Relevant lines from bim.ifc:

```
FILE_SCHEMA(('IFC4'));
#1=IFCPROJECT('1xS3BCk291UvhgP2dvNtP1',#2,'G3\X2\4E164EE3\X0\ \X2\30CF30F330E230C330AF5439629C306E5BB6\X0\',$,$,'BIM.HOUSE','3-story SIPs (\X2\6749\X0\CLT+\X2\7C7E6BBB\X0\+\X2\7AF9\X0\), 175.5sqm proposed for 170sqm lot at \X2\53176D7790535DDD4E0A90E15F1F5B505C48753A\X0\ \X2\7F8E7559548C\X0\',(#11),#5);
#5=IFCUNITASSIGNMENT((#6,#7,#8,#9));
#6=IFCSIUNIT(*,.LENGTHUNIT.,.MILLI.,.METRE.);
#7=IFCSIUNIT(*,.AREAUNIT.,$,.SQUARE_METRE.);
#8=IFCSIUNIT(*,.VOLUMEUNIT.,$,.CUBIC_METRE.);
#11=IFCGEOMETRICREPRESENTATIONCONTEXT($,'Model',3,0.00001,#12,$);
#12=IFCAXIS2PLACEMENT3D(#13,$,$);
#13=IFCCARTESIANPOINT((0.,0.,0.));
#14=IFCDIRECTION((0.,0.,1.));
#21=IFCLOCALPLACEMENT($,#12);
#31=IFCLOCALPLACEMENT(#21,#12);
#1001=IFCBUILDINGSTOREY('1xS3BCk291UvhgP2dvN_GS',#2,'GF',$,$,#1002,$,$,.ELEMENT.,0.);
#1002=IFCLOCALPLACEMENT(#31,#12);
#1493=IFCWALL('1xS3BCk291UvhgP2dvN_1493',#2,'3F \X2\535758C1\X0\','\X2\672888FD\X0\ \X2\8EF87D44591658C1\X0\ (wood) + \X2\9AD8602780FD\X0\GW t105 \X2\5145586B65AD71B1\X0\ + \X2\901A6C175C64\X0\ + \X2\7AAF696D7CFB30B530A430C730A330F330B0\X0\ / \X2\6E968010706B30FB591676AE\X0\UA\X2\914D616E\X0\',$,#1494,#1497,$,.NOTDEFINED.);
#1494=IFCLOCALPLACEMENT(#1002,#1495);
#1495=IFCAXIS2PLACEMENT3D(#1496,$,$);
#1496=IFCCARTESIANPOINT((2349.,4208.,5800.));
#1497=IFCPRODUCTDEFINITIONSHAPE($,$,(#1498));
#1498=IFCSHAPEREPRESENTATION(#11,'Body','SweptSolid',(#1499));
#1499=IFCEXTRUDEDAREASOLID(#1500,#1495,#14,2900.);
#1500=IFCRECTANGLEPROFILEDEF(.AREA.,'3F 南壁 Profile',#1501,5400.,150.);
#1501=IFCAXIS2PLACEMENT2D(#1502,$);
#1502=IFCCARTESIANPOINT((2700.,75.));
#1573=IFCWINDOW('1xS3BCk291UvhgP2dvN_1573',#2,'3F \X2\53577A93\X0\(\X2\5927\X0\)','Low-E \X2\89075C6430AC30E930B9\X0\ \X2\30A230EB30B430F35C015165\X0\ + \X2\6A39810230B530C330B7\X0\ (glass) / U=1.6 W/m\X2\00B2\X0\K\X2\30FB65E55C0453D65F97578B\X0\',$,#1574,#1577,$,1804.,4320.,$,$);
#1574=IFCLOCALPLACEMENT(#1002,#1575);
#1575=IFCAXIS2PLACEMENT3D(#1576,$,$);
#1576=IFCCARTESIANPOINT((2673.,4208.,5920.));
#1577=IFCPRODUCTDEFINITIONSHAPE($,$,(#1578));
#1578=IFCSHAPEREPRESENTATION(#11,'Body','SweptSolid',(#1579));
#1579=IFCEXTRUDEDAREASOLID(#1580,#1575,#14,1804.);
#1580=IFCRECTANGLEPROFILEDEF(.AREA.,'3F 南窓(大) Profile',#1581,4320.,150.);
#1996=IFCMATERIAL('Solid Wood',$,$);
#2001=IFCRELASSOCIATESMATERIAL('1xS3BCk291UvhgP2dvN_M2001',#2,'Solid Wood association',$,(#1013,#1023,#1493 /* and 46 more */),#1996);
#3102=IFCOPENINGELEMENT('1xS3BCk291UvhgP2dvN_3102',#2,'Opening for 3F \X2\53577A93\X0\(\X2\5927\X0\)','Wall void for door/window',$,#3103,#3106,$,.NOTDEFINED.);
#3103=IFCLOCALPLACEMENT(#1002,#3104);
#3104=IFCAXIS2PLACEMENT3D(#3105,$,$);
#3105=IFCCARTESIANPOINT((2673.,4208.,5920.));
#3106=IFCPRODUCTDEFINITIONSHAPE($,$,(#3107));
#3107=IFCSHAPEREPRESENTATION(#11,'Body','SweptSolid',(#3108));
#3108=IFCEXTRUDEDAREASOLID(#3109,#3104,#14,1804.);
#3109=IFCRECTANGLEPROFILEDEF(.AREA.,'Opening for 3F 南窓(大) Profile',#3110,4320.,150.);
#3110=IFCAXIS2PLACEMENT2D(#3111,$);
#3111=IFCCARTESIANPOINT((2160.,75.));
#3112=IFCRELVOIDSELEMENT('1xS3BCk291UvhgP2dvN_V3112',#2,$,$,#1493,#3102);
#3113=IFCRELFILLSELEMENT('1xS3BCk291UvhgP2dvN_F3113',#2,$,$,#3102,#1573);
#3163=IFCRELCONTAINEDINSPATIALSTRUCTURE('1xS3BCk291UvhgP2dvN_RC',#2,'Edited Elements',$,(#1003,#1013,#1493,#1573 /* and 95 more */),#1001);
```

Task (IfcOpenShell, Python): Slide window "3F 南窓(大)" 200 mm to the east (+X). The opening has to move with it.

```python
import ifcopenshell
import ifcopenshell.api.geometry
import ifcopenshell.util.placement
import ifcopenshell.util.unit

model = ifcopenshell.open("bim.ifc")
unit_scale = ifcopenshell.util.unit.calculate_unit_scale(model)

window = model.by_guid("1xS3BCk291UvhgP2dvN_1573")
opening = window.FillsVoids[0].RelatingOpeningElement
wall = opening.VoidsElements[0].RelatingBuildingElement

wall_matrix = ifcopenshell.util.placement.get_local_placement(wall.ObjectPlacement)
shift = wall_matrix[:3, 0] * 0.2 / unit_scale
before = ifcopenshell.util.placement.get_local_placement(window.ObjectPlacement)[:3, 3].copy()

# The window is not placed relative to its opening, so move both.
for product in (opening, window):
    matrix = ifcopenshell.util.placement.get_local_placement(product.ObjectPlacement)
    matrix[:3, 3] += shift
    ifcopenshell.api.geometry.edit_object_placement(model, product=product, matrix=matrix, is_si=False)

after = ifcopenshell.util.placement.get_local_placement(window.ObjectPlacement)[:3, 3]
print("window moved by", (after - before).round(3) + 0.0)

model.write("bim_edited.ifc")
```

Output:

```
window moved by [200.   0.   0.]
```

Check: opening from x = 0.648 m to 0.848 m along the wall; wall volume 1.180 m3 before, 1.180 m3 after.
